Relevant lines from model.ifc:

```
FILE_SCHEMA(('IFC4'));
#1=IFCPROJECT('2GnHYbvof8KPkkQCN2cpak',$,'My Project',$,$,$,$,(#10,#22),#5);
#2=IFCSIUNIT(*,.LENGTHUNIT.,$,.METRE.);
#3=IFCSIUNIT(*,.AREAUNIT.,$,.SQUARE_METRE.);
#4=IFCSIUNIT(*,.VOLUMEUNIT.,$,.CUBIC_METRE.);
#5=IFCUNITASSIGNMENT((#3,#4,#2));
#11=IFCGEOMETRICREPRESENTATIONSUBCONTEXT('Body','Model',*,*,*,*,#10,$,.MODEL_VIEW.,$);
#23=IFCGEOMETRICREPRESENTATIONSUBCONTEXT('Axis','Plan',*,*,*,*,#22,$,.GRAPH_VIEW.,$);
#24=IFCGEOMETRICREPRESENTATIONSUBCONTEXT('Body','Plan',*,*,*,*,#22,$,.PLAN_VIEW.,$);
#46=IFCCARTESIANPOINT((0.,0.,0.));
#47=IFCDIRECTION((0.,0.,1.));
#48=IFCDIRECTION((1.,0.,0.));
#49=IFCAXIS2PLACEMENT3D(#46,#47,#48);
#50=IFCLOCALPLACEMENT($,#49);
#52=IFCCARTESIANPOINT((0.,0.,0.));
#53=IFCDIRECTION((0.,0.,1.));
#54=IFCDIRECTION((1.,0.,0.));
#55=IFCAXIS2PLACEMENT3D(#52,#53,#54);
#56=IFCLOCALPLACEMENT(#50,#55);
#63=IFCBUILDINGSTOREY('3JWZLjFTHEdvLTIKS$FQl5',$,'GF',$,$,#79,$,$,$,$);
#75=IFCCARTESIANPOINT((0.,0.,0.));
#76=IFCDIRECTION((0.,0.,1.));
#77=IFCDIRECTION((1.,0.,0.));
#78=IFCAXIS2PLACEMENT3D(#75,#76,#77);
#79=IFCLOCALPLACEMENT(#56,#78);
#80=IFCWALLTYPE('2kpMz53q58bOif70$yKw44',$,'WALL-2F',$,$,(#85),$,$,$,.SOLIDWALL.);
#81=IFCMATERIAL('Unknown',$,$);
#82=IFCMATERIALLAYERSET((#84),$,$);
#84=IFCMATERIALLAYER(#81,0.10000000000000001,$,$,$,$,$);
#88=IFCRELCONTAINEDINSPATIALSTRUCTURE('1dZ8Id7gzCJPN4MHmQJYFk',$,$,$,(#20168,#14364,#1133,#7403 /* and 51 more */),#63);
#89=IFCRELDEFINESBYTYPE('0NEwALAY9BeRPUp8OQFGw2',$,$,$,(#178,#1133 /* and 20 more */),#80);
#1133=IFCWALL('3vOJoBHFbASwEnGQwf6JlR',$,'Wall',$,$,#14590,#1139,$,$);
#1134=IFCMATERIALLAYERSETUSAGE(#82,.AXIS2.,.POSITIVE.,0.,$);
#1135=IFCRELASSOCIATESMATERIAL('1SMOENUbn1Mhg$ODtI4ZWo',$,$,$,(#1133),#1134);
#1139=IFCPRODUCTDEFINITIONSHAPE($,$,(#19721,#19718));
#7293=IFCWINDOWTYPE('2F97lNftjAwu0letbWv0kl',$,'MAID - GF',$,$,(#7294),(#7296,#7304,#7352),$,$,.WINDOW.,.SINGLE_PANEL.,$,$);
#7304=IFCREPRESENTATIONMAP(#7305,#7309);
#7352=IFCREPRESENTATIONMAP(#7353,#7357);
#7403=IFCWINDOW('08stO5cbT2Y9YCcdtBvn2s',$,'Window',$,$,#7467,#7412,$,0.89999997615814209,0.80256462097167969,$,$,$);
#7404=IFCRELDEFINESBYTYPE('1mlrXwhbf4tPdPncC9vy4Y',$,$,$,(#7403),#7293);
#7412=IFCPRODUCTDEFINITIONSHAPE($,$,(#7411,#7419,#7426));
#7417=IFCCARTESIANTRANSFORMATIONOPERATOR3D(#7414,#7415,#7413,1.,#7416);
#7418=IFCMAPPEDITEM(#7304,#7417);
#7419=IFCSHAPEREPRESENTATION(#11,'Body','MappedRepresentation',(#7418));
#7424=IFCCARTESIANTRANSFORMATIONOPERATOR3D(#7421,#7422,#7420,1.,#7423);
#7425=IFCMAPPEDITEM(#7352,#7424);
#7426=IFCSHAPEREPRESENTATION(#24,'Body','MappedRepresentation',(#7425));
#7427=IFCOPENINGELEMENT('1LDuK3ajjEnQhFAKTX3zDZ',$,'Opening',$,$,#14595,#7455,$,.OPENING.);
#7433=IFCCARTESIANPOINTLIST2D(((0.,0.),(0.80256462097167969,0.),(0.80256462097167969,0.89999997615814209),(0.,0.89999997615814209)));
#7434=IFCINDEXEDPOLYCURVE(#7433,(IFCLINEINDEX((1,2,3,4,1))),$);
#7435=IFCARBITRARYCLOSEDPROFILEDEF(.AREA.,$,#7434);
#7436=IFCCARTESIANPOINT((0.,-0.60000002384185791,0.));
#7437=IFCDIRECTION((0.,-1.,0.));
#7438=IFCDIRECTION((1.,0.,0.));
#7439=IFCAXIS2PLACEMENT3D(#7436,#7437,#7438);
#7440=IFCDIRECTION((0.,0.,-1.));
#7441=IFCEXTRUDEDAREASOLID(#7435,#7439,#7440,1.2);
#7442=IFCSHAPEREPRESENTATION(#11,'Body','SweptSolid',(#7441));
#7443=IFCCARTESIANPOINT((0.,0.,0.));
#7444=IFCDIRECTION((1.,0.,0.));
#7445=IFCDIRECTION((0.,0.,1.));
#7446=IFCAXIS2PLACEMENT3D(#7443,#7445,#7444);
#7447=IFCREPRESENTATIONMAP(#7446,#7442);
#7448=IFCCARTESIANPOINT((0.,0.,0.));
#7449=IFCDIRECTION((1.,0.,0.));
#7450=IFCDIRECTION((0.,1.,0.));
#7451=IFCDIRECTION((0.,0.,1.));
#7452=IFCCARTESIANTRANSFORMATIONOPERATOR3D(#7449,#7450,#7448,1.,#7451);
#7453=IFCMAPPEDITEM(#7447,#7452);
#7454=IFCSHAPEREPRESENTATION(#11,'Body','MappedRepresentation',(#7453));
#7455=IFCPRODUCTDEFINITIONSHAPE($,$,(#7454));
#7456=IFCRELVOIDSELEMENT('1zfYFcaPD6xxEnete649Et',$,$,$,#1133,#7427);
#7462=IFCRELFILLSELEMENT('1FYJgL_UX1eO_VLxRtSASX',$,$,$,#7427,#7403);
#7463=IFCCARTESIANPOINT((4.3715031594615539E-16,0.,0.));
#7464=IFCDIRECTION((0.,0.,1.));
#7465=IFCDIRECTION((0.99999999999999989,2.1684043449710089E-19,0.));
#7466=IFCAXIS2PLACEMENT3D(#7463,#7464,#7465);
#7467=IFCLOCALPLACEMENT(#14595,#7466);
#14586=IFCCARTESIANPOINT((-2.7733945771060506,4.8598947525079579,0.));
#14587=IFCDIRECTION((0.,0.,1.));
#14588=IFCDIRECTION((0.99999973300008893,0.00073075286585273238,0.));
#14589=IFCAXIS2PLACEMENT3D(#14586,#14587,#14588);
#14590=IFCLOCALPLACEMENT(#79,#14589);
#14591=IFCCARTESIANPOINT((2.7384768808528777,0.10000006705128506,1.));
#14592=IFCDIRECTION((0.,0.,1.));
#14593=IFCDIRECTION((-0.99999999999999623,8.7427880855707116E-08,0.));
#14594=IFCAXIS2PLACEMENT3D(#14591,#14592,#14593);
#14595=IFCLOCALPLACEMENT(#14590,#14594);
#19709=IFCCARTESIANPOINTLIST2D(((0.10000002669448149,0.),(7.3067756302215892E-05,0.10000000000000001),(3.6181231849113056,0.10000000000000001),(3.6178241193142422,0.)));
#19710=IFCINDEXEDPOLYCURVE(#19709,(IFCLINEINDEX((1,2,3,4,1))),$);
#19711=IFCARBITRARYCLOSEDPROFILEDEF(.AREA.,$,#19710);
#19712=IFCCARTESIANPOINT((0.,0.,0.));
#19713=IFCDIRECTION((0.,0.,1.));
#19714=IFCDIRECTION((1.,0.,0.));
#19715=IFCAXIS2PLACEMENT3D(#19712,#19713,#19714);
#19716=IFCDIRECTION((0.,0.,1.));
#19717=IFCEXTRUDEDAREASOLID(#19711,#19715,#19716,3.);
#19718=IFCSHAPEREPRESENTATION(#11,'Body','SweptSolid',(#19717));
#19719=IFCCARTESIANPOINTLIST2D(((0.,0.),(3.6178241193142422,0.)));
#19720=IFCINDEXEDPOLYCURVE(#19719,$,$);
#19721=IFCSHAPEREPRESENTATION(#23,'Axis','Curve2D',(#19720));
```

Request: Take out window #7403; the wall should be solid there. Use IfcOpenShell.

```python
import ifcopenshell
import ifcopenshell.api.feature
import ifcopenshell.api.root
import ifcopenshell.geom
import ifcopenshell.util.shape

model = ifcopenshell.open("model.ifc")
settings = ifcopenshell.geom.settings()


def volume(element):
    """Net volume in cubic metres, openings subtracted."""
    shape = ifcopenshell.geom.create_shape(settings, element)
    return ifcopenshell.util.shape.get_volume(shape.geometry)


window = model.by_guid("08stO5cbT2Y9YCcdtBvn2s")
opening = window.FillsVoids[0].RelatingOpeningElement
wall = opening.VoidsElements[0].RelatingBuildingElement
before = volume(wall)

ifcopenshell.api.root.remove_product(model, product=window)
ifcopenshell.api.feature.remove_feature(model, feature=opening)

after = volume(wall)

print(f"wall volume {before:.3f} -> {after:.3f} m3")

model.write("model_updated.ifc")
```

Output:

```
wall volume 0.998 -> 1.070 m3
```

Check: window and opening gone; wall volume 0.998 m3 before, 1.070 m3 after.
